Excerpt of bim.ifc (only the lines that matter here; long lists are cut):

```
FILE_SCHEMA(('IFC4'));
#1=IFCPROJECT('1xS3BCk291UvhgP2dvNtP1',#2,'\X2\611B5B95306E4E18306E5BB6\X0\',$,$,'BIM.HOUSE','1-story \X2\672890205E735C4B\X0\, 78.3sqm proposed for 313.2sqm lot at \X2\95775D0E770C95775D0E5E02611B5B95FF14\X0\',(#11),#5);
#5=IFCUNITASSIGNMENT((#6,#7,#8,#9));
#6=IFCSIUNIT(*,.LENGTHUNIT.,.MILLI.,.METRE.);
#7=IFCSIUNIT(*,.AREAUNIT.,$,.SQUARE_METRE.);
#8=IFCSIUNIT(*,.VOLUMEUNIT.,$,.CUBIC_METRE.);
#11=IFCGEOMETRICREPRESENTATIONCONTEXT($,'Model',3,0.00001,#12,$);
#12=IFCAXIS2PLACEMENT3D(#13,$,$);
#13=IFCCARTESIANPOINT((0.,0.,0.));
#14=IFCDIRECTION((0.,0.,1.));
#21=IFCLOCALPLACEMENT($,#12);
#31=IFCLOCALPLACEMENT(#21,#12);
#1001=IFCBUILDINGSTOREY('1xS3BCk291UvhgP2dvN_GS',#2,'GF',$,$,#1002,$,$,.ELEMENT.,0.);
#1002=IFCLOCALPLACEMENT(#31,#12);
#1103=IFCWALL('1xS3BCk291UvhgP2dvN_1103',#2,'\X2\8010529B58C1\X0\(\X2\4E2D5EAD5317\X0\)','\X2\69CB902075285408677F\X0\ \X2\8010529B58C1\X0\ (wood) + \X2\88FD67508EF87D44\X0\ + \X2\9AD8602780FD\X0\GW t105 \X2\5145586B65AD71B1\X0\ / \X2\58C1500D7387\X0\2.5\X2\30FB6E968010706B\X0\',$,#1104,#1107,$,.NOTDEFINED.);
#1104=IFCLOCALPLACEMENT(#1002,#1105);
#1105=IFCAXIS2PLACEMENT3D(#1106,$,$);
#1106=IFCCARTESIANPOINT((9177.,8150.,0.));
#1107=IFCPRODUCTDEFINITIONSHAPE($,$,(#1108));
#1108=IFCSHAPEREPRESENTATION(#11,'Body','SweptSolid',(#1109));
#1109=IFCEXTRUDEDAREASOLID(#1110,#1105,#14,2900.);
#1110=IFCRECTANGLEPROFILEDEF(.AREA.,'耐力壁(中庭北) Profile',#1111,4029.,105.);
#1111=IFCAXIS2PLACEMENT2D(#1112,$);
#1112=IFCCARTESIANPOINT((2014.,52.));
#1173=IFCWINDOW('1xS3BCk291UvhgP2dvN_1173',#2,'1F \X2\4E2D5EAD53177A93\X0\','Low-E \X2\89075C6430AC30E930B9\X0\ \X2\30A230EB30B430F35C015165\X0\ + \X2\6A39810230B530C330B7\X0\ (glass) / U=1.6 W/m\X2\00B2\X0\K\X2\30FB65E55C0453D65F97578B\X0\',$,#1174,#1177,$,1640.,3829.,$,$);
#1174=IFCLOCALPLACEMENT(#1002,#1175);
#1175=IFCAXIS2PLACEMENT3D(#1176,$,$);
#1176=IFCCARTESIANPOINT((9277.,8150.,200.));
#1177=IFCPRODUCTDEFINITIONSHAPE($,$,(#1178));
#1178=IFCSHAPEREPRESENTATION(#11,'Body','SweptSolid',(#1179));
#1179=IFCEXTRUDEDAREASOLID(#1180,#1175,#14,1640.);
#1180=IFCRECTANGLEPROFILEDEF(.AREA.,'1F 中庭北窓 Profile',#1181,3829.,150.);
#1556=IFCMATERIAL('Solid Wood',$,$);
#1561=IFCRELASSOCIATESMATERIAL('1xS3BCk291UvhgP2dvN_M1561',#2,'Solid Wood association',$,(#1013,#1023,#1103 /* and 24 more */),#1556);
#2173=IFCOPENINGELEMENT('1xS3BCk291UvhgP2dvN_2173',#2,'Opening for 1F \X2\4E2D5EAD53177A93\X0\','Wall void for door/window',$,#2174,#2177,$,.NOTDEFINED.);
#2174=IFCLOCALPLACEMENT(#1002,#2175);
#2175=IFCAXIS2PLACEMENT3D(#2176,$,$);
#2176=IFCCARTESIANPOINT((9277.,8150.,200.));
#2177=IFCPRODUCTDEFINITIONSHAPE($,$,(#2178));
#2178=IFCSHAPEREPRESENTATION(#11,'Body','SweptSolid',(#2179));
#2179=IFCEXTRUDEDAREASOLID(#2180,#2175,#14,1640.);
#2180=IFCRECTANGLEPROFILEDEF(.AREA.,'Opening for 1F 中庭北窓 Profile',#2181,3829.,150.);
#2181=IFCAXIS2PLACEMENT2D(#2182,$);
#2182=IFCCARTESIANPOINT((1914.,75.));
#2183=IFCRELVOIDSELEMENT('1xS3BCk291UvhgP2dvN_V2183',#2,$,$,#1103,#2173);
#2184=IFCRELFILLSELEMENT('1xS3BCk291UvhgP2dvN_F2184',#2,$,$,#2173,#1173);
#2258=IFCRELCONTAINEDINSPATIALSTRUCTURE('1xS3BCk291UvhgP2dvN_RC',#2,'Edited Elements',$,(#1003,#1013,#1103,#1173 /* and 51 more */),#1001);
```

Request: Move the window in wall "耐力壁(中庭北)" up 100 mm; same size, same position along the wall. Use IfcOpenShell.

```python
import numpy as np
import ifcopenshell
import ifcopenshell.api.geometry
import ifcopenshell.util.placement
import ifcopenshell.util.unit

model = ifcopenshell.open("bim.ifc")
unit_scale = ifcopenshell.util.unit.calculate_unit_scale(model)

window = model.by_guid("1xS3BCk291UvhgP2dvN_1173")
opening = window.FillsVoids[0].RelatingOpeningElement
dz = 0.1 / unit_scale

shift = np.array([0.0, 0.0, dz])
# The window is not placed relative to its opening, so move both.
for product in (opening, window):
    matrix = ifcopenshell.util.placement.get_local_placement(product.ObjectPlacement)
    matrix[:3, 3] += shift
    ifcopenshell.api.geometry.edit_object_placement(model, product=product, matrix=matrix, is_si=False)

print(f"moved by {dz * unit_scale:+.3f} m")

model.write("bim_updated.ifc")
```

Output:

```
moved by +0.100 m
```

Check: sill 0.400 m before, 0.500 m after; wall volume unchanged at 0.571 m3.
